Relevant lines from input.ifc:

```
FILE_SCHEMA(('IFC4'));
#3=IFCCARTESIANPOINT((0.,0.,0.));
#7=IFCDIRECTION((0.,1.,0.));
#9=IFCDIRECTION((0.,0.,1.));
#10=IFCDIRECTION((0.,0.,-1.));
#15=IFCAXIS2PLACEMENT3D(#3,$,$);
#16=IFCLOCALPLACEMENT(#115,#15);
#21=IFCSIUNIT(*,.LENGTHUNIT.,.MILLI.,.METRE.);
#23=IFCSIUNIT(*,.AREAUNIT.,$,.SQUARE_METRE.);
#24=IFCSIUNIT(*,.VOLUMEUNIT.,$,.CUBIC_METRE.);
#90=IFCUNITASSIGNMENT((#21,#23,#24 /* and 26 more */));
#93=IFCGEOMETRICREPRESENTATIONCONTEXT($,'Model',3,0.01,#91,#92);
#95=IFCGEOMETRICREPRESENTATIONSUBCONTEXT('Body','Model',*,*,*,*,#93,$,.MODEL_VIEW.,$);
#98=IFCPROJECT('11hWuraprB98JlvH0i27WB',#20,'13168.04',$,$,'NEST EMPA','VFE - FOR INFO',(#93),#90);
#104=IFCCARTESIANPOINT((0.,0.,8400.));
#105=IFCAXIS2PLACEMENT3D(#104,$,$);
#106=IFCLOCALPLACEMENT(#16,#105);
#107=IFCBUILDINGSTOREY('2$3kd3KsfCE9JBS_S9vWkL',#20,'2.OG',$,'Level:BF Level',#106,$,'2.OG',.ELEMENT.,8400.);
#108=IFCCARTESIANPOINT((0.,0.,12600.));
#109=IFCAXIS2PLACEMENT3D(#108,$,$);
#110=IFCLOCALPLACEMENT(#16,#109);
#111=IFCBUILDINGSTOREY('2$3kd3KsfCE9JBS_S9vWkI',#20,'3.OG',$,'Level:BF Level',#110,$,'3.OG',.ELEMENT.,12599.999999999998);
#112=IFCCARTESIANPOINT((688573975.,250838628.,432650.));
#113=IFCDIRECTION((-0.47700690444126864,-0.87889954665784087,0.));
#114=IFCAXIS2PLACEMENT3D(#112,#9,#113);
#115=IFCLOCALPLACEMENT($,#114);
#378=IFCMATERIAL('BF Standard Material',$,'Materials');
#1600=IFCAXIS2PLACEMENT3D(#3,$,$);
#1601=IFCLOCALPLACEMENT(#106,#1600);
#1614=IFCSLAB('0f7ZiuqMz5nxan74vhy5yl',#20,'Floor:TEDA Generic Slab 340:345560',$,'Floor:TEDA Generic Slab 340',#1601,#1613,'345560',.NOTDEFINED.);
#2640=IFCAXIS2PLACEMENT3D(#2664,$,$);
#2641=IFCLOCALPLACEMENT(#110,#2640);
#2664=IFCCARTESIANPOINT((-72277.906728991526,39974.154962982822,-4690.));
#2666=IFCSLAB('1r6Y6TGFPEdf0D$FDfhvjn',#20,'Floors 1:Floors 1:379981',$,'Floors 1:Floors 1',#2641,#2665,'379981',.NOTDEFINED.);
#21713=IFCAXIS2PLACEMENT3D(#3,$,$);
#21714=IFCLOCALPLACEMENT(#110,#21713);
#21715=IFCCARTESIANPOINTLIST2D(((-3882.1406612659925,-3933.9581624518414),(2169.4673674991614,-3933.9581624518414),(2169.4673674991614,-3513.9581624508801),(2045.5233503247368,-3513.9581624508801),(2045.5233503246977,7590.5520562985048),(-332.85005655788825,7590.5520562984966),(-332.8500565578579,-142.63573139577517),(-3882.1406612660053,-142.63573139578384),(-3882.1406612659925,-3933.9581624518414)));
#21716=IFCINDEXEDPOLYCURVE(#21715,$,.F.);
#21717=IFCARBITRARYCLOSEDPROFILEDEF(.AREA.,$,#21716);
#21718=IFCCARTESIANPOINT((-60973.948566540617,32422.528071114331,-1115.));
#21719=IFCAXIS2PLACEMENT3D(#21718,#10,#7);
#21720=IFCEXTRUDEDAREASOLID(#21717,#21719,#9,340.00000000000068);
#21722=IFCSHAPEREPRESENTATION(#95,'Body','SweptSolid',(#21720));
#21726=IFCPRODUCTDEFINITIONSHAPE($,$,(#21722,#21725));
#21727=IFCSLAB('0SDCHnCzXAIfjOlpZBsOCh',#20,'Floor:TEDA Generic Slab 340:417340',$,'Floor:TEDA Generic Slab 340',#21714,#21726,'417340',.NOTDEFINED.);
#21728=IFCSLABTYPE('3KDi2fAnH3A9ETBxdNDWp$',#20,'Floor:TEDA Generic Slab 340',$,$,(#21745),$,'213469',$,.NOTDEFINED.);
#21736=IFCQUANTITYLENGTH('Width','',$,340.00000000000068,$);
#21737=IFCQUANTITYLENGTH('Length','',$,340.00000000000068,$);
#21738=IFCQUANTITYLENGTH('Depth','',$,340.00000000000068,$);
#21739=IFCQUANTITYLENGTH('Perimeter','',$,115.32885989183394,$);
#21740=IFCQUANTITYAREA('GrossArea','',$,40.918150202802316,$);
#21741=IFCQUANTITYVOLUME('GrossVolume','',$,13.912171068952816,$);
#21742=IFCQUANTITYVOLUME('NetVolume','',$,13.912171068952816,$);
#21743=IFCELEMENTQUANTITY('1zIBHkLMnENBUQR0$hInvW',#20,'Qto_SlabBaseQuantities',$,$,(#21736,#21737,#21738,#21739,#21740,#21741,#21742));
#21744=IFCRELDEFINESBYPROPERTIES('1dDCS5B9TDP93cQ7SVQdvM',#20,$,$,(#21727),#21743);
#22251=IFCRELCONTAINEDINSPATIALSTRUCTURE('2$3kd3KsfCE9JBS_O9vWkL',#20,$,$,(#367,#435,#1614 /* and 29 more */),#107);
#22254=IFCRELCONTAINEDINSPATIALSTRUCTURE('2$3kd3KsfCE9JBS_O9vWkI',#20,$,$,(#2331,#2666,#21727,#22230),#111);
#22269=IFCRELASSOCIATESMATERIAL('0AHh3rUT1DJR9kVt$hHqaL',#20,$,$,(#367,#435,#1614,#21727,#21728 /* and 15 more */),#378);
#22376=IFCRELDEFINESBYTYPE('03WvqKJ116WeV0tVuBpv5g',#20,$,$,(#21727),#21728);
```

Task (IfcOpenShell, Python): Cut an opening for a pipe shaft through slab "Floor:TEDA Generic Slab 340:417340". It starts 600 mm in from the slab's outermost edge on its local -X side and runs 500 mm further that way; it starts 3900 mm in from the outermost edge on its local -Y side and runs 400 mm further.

```python
import numpy as np
import ifcopenshell
import ifcopenshell.api.feature
import ifcopenshell.api.geometry
import ifcopenshell.api.pset
import ifcopenshell.api.root
import ifcopenshell.geom
import ifcopenshell.util.element
import ifcopenshell.util.placement
import ifcopenshell.util.representation
import ifcopenshell.util.shape
import ifcopenshell.util.unit

model = ifcopenshell.open("input.ifc")
unit_scale = ifcopenshell.util.unit.calculate_unit_scale(model)
volume_scale = ifcopenshell.util.unit.calculate_unit_scale(model, "VOLUMEUNIT")
settings = ifcopenshell.geom.settings()


def volume(element):
    """Net volume in cubic metres, openings subtracted."""
    shape = ifcopenshell.geom.create_shape(settings, element)
    return ifcopenshell.util.shape.get_volume(shape.geometry)


slab = model.by_guid("0SDCHnCzXAIfjOlpZBsOCh")
before = volume(slab)

# Extent in the slab's own axes, in metres. The edges named are its -X and -Y sides.
slab_shape = ifcopenshell.geom.create_shape(settings, slab)
vertices = ifcopenshell.util.shape.get_vertices(slab_shape.geometry)
x_min, y_min, bottom = vertices.min(axis=0)
top = vertices[:, 2].max()

opening = ifcopenshell.api.root.create_entity(model, ifc_class="IfcOpeningElement", name="Pipe shaft opening", predefined_type="OPENING")
context = ifcopenshell.util.representation.get_context(model, "Model", "Body", "MODEL_VIEW")
width, depth = 0.5, 0.4
outline = [(0.0, 0.0), (width, 0.0), (width, depth), (0.0, depth), (0.0, 0.0)]
# Overshoot both faces by 50 mm so the cut is clean.
shape = ifcopenshell.api.geometry.add_slab_representation(
    model, context=context, depth=top - bottom + 0.1, polyline=outline
)
ifcopenshell.api.geometry.assign_representation(model, product=opening, representation=shape)

matrix = ifcopenshell.util.placement.get_local_placement(slab.ObjectPlacement)
matrix[:, 3] = matrix @ np.append(np.array([x_min + 0.6, y_min + 3.9, bottom - 0.05]) / unit_scale, 1.0)
ifcopenshell.api.geometry.edit_object_placement(model, product=opening, matrix=matrix, is_si=False)
ifcopenshell.api.feature.add_feature(model, feature=opening, element=slab)

after = volume(slab)

# Update the slab's stored quantities.
qto = model.by_id(ifcopenshell.util.element.get_pset(slab, "Qto_SlabBaseQuantities", should_inherit=False)["id"])
ifcopenshell.api.pset.edit_qto(model, qto=qto, properties={"NetVolume": after / volume_scale})

print(f"slab volume {before:.3f} -> {after:.3f} m3")

model.write("input_v2.ifc")
```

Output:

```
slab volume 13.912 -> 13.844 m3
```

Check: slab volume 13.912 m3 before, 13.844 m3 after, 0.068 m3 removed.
